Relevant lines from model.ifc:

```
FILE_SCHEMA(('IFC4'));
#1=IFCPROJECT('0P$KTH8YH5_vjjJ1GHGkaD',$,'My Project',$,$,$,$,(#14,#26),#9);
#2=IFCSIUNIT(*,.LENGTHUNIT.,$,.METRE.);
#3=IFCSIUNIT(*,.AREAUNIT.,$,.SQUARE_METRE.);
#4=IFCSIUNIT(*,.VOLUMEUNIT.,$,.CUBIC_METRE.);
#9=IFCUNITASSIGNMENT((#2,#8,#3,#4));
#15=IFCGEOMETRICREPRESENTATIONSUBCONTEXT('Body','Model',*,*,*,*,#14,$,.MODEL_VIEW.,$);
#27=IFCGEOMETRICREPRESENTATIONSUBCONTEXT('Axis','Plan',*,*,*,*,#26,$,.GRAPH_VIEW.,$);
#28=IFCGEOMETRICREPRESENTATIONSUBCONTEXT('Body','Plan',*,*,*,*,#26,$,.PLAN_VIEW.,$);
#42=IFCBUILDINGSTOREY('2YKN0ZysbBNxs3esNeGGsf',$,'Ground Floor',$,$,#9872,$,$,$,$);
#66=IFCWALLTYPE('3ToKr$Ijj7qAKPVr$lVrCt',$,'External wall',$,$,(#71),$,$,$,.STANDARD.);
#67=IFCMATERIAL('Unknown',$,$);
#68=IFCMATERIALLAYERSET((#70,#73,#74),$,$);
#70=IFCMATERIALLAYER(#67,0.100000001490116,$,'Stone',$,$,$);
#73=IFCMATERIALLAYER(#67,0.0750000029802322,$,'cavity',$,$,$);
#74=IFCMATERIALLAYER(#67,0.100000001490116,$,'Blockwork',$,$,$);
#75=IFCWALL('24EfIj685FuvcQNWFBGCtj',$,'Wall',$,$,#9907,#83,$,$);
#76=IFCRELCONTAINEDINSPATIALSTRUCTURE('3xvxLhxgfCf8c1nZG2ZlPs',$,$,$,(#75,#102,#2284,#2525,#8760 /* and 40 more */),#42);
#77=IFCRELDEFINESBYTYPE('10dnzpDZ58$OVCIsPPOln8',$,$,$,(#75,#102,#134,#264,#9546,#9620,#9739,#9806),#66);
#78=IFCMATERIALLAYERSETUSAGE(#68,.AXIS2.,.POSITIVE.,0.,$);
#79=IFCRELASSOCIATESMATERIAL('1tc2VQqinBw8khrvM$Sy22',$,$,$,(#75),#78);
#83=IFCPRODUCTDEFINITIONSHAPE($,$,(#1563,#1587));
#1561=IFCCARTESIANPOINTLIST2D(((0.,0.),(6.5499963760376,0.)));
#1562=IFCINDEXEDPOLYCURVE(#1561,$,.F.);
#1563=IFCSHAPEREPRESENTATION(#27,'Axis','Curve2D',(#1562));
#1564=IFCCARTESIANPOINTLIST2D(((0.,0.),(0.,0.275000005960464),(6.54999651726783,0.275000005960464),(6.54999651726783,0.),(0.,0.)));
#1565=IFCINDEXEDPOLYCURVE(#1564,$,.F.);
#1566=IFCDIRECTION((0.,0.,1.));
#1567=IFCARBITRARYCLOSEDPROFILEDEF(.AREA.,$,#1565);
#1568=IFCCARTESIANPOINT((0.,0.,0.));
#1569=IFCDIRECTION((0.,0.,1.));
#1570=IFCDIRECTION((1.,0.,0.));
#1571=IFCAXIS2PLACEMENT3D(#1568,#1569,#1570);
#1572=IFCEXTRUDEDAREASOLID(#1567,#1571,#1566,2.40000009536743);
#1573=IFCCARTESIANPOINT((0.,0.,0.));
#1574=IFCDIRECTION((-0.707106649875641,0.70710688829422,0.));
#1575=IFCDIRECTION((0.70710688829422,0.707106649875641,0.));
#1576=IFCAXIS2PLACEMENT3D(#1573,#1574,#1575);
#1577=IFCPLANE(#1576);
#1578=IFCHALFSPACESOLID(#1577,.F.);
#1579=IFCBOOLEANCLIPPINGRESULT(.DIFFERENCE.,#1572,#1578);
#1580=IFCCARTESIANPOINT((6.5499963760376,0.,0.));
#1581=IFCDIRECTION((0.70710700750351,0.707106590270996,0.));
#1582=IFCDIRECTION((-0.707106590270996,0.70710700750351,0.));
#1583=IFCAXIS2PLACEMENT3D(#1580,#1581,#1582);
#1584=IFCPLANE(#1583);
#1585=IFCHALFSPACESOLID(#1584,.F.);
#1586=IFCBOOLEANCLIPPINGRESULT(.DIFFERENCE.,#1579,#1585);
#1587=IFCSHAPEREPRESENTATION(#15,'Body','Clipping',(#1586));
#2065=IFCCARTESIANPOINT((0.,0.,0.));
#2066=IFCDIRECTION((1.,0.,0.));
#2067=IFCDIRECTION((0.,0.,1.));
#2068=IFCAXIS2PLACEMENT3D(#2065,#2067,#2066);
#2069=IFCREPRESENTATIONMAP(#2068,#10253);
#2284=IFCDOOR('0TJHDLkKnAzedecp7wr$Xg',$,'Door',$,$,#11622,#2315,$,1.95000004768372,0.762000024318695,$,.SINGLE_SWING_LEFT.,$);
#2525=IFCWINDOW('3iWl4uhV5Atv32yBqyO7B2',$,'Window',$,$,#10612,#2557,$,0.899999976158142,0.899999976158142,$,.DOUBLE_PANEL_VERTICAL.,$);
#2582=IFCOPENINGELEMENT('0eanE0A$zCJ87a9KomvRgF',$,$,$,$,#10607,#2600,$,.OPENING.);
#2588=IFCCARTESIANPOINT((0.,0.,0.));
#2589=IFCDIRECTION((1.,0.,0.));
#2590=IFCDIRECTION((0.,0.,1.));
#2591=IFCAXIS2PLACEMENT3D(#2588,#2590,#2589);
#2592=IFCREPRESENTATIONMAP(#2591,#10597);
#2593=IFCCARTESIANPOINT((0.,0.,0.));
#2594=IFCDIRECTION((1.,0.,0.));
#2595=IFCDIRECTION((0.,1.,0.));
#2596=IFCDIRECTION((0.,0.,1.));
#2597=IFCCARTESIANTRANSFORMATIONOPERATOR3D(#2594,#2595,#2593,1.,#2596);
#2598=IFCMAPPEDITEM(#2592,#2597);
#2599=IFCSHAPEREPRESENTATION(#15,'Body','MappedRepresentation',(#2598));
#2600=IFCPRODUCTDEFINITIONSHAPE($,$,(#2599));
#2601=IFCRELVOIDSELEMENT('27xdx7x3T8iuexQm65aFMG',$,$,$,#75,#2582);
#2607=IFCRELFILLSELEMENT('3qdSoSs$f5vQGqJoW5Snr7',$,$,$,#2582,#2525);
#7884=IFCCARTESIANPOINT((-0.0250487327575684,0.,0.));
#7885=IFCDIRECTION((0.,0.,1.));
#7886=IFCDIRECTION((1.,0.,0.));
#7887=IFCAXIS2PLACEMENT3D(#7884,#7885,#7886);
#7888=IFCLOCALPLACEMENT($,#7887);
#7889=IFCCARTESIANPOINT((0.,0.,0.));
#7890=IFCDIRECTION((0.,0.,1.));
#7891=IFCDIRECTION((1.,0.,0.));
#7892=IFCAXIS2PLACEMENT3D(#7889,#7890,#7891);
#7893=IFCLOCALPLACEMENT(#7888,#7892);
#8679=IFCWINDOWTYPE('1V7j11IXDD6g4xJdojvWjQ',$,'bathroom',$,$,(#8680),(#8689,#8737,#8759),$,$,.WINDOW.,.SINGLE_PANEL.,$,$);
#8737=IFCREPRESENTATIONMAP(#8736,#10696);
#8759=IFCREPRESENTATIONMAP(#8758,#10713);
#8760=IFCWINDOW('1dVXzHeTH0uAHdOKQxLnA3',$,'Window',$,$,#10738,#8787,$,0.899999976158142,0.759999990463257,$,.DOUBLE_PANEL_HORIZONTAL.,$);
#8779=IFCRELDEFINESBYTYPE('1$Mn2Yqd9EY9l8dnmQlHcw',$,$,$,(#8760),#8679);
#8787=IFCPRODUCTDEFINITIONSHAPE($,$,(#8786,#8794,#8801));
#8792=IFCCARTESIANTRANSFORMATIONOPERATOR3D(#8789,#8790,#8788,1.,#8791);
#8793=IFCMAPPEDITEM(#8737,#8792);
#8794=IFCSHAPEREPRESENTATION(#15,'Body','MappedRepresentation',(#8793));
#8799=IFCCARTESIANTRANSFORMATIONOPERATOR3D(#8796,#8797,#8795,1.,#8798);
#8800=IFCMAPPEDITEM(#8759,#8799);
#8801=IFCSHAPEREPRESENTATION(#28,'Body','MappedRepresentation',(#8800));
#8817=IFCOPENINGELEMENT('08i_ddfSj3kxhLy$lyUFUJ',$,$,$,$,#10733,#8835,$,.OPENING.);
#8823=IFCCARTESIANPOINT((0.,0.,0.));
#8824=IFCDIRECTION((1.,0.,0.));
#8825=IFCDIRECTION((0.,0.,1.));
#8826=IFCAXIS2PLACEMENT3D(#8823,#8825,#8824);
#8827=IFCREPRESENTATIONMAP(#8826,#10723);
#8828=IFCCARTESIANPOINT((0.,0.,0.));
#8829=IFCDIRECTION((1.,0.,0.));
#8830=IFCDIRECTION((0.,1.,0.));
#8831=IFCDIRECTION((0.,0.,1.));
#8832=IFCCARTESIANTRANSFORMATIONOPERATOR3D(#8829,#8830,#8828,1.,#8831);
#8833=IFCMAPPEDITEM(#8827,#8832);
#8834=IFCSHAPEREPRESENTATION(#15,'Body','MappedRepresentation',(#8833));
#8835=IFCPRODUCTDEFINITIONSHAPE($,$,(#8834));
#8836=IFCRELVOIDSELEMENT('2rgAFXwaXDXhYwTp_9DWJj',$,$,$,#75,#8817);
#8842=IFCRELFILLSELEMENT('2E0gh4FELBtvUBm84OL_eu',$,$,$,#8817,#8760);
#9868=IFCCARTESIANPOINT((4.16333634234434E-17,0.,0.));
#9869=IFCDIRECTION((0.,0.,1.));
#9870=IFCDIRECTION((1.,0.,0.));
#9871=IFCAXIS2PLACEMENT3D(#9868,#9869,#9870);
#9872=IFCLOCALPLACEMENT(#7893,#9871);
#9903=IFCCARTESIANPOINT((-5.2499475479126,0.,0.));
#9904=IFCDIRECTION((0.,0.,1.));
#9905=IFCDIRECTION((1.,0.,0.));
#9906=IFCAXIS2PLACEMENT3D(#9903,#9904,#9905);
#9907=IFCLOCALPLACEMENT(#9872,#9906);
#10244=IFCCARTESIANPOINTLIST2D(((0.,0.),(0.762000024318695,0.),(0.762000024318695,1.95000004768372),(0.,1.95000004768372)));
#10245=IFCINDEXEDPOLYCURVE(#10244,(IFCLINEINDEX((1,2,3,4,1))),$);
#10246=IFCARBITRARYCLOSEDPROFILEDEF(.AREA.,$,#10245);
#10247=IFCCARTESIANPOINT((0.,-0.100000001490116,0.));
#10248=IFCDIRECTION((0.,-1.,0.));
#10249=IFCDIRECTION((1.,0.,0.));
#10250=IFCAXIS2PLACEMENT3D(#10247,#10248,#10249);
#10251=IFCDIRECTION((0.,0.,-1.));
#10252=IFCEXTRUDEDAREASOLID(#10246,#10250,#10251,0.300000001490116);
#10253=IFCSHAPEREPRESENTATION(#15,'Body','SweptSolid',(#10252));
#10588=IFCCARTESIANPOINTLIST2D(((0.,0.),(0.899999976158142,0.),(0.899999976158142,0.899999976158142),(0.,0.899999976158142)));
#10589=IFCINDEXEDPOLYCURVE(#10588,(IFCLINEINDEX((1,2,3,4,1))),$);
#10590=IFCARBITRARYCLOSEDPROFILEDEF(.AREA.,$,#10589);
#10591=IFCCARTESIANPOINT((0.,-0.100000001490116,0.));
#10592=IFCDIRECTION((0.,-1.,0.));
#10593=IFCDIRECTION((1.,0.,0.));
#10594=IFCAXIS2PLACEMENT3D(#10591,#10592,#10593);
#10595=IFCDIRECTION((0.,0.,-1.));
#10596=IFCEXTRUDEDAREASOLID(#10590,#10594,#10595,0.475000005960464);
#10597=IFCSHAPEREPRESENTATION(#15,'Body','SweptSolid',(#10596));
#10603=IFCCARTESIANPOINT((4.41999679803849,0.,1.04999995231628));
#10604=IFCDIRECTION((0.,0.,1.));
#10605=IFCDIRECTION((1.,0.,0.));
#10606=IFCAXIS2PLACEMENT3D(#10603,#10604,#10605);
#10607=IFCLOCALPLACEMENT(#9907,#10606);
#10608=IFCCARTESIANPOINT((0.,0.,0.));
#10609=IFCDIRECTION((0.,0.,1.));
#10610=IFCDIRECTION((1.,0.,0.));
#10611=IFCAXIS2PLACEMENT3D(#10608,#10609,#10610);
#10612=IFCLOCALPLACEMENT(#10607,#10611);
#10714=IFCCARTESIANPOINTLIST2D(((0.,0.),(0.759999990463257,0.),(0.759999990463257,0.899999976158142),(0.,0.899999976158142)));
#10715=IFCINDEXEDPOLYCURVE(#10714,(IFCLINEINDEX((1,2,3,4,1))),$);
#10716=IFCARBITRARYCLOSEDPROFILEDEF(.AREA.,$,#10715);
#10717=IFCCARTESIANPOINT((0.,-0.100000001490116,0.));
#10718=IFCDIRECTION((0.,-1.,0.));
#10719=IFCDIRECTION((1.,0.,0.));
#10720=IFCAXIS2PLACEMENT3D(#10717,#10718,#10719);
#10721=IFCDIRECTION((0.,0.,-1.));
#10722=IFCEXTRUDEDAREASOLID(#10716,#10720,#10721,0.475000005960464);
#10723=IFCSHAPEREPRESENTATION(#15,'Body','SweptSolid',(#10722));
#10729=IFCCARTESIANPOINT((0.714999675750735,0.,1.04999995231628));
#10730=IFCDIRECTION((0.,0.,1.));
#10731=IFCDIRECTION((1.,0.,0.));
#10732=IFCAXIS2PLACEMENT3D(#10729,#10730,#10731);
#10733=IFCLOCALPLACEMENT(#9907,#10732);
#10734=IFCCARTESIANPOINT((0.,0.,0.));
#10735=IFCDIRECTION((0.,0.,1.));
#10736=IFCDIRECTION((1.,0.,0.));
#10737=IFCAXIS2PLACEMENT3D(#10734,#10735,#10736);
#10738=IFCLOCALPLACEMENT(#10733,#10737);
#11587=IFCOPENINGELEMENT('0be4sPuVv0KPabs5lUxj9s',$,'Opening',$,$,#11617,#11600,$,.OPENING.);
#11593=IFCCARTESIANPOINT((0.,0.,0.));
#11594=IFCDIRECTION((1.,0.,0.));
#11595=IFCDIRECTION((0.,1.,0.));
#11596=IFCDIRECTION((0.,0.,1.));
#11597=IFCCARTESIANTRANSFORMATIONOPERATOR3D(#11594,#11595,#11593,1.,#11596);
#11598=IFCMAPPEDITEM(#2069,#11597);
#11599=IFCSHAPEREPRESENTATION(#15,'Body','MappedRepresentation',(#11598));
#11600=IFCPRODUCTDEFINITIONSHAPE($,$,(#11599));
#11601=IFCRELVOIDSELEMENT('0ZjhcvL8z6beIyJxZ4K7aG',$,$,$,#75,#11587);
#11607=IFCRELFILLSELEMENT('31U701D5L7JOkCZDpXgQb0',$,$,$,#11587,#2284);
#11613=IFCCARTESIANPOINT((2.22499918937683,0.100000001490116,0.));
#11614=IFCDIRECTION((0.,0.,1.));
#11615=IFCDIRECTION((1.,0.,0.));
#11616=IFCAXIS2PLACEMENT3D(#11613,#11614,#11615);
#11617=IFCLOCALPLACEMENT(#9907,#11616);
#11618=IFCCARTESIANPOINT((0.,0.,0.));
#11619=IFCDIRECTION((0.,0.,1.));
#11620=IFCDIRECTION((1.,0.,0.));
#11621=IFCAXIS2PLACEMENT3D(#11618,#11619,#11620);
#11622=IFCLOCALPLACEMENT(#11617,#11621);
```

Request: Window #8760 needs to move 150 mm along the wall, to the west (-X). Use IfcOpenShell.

```python
import ifcopenshell
import ifcopenshell.api.geometry
import ifcopenshell.util.placement

model = ifcopenshell.open("model.ifc")

window = model.by_guid("1dVXzHeTH0uAHdOKQxLnA3")
opening = window.FillsVoids[0].RelatingOpeningElement
wall = opening.VoidsElements[0].RelatingBuildingElement

wall_matrix = ifcopenshell.util.placement.get_local_placement(wall.ObjectPlacement)
shift = wall_matrix[:3, 0] * -0.15
before = ifcopenshell.util.placement.get_local_placement(window.ObjectPlacement)[:3, 3].copy()

# The window is placed relative to its opening, so it follows when the opening moves.
matrix = ifcopenshell.util.placement.get_local_placement(opening.ObjectPlacement)
matrix[:3, 3] += shift
ifcopenshell.api.geometry.edit_object_placement(
    model, product=opening, matrix=matrix, is_si=False, should_transform_children=True
)

after = ifcopenshell.util.placement.get_local_placement(window.ObjectPlacement)[:3, 3]
print("window moved by", (after - before).round(3) + 0.0)

model.write("model_updated.ifc")
```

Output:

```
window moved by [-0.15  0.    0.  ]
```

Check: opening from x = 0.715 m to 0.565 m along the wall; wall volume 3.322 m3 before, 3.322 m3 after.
